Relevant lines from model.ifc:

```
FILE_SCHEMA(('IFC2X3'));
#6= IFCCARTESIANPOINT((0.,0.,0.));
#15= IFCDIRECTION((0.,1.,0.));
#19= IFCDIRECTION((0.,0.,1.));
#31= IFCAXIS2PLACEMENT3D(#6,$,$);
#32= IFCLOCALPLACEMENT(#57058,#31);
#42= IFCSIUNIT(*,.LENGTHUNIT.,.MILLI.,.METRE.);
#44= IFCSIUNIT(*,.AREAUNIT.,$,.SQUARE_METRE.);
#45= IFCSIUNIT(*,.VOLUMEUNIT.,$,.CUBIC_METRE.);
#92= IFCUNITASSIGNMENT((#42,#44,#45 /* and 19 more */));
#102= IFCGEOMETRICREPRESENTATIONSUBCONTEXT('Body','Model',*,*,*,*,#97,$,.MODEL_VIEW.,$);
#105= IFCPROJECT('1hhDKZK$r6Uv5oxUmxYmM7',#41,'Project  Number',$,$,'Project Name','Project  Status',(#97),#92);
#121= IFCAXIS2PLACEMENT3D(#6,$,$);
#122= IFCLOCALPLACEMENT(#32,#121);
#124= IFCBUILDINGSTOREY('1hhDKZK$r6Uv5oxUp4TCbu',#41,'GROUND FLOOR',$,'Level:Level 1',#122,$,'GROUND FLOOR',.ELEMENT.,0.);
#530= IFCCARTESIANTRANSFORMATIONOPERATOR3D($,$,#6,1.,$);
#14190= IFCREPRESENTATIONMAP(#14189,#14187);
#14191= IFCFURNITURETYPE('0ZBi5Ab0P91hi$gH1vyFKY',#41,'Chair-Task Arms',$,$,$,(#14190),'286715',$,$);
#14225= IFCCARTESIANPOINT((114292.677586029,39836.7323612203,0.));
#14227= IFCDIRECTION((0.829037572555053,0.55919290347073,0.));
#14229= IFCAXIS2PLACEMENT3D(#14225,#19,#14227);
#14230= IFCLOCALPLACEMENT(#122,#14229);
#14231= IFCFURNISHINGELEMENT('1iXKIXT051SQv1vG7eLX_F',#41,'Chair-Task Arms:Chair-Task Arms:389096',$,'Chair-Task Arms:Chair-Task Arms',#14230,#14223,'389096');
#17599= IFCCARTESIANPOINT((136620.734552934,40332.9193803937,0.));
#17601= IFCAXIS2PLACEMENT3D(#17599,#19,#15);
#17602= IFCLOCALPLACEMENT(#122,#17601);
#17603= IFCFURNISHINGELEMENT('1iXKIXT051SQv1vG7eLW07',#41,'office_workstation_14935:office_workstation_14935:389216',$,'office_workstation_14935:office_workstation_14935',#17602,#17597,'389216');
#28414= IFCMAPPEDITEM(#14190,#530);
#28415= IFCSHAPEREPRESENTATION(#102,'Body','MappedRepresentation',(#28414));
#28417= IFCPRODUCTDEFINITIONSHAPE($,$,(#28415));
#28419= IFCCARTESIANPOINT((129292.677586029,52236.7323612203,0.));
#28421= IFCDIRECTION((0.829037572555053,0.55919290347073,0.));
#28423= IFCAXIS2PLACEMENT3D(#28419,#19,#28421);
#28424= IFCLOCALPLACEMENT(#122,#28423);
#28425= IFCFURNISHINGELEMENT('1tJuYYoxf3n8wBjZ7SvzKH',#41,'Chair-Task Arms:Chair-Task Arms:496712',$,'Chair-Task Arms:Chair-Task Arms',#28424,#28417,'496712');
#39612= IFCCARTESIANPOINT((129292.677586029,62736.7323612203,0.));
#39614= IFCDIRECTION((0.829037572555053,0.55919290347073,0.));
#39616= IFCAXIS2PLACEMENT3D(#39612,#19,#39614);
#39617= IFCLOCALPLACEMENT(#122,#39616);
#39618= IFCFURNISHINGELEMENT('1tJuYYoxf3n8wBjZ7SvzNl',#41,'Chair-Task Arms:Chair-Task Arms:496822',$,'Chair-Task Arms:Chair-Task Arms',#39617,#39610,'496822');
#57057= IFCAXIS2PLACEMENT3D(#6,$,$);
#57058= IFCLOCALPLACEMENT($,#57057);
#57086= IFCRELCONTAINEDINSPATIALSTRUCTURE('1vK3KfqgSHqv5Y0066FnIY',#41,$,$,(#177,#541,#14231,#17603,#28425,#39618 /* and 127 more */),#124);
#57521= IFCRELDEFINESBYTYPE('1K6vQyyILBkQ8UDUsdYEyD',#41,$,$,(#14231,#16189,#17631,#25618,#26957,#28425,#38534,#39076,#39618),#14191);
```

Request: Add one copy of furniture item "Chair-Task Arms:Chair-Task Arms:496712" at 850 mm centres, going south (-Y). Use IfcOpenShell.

```python
import numpy as np
import ifcopenshell
import ifcopenshell.api.geometry
import ifcopenshell.api.root
import ifcopenshell.util.element
import ifcopenshell.util.placement

model = ifcopenshell.open("model.ifc")


def reuse_history(source, copy):
    """copy_class also copies each property set's owner history, people and application; keep the originals."""
    for rel in copy.IsDefinedBy:
        if rel.is_a("IfcRelDefinesByProperties") and (history := rel.RelatingPropertyDefinition.OwnerHistory):
            rel.RelatingPropertyDefinition.OwnerHistory = source.OwnerHistory
            ifcopenshell.util.element.remove_deep2(model, history)


source = model.by_guid("1tJuYYoxf3n8wBjZ7SvzKH")
base = ifcopenshell.util.placement.get_local_placement(source.ObjectPlacement)
step = np.array([0.0, -1.0, 0.0]) * 850.0

for i in range(1, 2):
    copy = ifcopenshell.api.root.copy_class(model, product=source)
    copy.Representation = ifcopenshell.util.element.copy_deep(
        model, source.Representation, exclude=["IfcGeometricRepresentationContext", "IfcRepresentationMap"]
    )
    copy.Name = "Chair-Task Arms:Chair-Task Arms"
    copy.Tag = None
    reuse_history(source, copy)
    matrix = base.copy()
    matrix[:3, 3] += i * step
    print("added at", matrix[:3, 3].round(3) + 0.0)
    ifcopenshell.api.geometry.edit_object_placement(model, product=copy, matrix=matrix, is_si=False)

model.write("model_v2.ifc")
```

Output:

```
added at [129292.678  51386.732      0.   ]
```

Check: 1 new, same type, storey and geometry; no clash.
